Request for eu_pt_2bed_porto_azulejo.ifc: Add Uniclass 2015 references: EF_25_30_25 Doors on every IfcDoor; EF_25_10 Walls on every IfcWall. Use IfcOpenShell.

First a look at what the model holds.

```python
import ifcopenshell

model = ifcopenshell.open("eu_pt_2bed_porto_azulejo.ifc")
print(model.schema)
print("classifications:", [c.Name for c in model.by_type("IfcClassification")])
for ifc_class in ("IfcDoor", "IfcRoof", "IfcStair", "IfcWall", "IfcWindow"):
    print(ifc_class, len(model.by_type(ifc_class)))
```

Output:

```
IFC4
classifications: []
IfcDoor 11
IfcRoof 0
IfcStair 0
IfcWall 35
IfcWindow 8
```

```python
import ifcopenshell
import ifcopenshell.api.classification

model = ifcopenshell.open("eu_pt_2bed_porto_azulejo.ifc")

system = ifcopenshell.api.classification.add_classification(model, classification="Uniclass 2015")

codes = {
    "IfcDoor": ("EF_25_30_25", "Doors"),
    "IfcWall": ("EF_25_10", "Walls"),
}
for ifc_class, (code, name) in codes.items():
    products = model.by_type(ifc_class)
    ifcopenshell.api.classification.add_reference(
        model, products=products, classification=system, identification=code, name=name
    )
    print(code, len(products))

model.write("eu_pt_2bed_porto_azulejo_rev.ifc")
```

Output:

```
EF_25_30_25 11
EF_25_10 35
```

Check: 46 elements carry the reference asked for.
